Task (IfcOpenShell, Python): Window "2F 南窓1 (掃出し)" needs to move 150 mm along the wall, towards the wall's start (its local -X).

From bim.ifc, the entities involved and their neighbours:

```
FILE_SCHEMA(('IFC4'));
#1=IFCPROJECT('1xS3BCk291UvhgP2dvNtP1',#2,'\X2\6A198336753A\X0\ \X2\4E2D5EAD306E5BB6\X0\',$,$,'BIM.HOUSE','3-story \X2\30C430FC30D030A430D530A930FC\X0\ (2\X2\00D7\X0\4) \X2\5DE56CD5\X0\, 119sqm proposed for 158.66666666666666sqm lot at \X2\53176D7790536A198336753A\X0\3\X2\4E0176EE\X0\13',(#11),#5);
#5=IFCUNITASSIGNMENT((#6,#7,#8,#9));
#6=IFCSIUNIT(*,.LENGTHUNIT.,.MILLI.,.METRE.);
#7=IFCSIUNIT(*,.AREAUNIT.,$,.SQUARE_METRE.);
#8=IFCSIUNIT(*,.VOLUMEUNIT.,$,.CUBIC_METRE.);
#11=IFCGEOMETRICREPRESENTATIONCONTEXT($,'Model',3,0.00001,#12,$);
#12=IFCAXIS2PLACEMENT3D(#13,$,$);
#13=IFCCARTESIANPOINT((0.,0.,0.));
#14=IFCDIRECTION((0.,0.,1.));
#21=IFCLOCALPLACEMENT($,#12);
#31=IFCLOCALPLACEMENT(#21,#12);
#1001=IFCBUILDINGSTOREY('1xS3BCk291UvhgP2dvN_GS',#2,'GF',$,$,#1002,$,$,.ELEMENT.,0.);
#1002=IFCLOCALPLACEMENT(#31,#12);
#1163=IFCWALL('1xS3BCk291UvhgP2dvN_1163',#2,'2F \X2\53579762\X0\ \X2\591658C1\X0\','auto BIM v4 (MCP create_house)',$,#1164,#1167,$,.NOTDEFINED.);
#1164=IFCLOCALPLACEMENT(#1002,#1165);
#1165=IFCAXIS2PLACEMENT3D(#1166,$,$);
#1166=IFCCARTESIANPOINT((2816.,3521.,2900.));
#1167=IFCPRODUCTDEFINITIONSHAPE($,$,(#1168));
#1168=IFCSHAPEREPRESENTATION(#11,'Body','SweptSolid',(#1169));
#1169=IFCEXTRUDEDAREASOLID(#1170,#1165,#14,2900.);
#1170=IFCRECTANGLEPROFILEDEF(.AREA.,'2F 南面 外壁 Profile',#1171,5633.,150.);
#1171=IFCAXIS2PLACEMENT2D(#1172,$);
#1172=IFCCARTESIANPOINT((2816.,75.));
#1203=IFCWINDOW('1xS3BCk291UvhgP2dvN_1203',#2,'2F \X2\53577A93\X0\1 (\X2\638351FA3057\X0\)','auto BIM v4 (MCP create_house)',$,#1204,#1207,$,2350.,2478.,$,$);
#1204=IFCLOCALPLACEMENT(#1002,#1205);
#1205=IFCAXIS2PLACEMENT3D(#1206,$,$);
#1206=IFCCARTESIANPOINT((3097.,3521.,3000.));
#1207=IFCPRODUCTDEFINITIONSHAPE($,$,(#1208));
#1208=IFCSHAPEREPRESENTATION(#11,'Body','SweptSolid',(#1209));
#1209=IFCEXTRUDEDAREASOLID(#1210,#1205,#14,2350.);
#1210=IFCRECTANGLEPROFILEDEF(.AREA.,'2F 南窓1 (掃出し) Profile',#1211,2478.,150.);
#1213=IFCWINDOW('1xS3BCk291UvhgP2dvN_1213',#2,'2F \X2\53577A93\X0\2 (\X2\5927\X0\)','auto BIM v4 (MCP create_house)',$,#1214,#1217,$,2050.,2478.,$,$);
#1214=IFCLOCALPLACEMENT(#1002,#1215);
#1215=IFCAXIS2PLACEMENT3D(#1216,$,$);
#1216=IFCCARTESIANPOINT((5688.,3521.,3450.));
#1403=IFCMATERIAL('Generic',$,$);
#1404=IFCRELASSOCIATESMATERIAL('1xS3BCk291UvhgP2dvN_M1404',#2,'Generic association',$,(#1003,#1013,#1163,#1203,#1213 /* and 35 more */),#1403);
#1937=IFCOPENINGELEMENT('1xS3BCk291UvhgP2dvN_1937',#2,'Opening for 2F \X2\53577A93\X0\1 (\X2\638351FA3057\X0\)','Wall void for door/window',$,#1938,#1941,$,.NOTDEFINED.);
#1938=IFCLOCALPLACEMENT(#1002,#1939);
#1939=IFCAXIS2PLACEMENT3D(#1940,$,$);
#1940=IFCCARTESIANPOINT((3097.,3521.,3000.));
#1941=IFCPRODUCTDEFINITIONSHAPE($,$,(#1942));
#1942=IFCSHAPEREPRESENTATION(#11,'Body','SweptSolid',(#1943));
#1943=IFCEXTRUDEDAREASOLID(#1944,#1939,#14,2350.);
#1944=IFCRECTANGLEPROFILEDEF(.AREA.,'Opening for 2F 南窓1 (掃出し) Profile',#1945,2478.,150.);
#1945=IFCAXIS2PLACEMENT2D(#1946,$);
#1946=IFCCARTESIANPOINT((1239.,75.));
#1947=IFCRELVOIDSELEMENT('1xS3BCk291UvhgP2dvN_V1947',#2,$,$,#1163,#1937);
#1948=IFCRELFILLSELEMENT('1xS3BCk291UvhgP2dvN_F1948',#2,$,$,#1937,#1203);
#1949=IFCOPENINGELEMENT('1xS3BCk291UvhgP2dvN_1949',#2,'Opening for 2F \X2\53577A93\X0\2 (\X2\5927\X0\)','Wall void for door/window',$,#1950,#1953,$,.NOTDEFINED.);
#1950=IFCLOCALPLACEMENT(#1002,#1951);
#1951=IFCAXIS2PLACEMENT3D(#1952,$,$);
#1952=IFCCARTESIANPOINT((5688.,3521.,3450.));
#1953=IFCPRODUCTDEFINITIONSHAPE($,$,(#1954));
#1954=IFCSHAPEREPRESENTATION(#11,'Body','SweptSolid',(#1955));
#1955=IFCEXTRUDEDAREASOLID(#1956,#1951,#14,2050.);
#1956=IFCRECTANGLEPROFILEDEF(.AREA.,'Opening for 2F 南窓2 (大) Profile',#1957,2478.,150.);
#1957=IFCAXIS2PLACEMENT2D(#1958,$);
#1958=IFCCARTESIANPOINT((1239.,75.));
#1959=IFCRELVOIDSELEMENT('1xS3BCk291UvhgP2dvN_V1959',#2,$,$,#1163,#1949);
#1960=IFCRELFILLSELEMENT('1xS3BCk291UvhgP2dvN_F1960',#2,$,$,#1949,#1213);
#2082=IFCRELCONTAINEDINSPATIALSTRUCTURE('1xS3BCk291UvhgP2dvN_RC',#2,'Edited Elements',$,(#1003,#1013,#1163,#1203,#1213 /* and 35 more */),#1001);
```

```python
import ifcopenshell
import ifcopenshell.api.geometry
import ifcopenshell.util.placement

model = ifcopenshell.open("bim.ifc")

window = model.by_guid("1xS3BCk291UvhgP2dvN_1203")
opening = window.FillsVoids[0].RelatingOpeningElement
wall = opening.VoidsElements[0].RelatingBuildingElement

wall_matrix = ifcopenshell.util.placement.get_local_placement(wall.ObjectPlacement)
shift = wall_matrix[:3, 0] * -150.0
before = ifcopenshell.util.placement.get_local_placement(window.ObjectPlacement)[:3, 3].copy()

# The window is not placed relative to its opening, so move both.
for product in (opening, window):
    matrix = ifcopenshell.util.placement.get_local_placement(product.ObjectPlacement)
    matrix[:3, 3] += shift
    ifcopenshell.api.geometry.edit_object_placement(model, product=product, matrix=matrix, is_si=False)

after = ifcopenshell.util.placement.get_local_placement(window.ObjectPlacement)[:3, 3]
print("window moved by", (after - before).round(3) + 0.0)

model.write("bim_edited.ifc")
```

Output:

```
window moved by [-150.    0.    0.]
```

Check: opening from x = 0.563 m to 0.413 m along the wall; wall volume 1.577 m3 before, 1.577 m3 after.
